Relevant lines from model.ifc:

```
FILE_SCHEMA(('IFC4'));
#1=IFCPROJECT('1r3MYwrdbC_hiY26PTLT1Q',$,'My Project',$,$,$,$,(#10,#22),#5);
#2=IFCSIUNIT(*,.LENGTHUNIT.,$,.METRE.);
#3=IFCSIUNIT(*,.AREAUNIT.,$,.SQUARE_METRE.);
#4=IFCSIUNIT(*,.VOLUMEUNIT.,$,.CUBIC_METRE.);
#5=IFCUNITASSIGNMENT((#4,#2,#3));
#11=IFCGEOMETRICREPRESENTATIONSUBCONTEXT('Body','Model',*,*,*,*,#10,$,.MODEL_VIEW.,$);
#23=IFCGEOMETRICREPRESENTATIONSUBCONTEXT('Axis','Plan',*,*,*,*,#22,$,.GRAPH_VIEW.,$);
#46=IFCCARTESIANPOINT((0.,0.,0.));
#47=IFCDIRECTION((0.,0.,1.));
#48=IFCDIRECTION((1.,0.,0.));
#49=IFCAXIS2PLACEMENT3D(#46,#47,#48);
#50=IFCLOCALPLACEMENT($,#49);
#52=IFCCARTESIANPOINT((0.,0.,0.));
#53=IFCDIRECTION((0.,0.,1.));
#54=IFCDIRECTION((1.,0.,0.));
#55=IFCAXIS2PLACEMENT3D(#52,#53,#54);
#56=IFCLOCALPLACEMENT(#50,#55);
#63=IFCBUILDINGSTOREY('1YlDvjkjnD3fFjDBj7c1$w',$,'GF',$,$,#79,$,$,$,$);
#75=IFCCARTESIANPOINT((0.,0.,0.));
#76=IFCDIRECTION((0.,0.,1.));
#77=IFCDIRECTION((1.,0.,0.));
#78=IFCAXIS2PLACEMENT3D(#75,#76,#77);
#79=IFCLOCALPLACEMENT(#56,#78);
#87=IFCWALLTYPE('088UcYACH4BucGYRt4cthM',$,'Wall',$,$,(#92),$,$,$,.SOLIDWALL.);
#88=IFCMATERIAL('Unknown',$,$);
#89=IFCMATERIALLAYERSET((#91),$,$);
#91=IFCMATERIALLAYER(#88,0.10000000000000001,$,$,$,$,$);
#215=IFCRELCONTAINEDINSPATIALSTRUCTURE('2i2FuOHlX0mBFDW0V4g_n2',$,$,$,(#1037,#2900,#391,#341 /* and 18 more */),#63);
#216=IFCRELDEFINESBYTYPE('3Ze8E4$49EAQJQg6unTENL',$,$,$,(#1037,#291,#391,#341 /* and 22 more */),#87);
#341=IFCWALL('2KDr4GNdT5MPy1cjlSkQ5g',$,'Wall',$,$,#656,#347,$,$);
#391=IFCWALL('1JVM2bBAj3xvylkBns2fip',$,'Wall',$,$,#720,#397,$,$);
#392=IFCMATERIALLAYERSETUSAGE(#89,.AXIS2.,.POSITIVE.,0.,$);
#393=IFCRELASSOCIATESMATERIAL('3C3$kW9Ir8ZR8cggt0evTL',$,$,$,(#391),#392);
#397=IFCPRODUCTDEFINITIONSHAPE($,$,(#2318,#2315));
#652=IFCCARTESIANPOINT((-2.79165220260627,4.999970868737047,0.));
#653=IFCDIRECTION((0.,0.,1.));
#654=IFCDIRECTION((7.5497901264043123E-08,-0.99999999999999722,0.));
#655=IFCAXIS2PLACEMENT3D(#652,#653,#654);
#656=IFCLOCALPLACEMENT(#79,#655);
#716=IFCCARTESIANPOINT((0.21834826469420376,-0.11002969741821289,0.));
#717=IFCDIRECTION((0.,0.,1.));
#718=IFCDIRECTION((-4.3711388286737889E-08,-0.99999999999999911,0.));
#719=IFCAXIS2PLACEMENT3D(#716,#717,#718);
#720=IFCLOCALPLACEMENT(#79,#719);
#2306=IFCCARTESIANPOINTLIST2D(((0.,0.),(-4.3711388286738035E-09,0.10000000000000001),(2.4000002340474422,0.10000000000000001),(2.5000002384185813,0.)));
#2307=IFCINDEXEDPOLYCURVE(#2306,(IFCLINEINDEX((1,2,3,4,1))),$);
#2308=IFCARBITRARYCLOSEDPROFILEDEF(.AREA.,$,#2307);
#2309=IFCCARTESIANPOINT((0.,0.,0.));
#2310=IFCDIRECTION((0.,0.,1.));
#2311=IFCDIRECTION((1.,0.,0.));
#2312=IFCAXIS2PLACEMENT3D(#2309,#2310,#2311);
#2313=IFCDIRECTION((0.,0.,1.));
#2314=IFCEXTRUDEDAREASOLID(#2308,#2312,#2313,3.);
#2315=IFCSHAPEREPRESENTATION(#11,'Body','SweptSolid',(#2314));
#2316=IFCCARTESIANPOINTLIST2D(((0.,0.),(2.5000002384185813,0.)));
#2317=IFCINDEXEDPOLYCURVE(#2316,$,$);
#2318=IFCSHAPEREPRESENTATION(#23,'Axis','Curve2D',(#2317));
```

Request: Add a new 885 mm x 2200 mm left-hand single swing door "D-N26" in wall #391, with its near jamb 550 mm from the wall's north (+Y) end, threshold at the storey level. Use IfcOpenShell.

```python
import numpy as np
import ifcopenshell
import ifcopenshell.api.feature
import ifcopenshell.api.geometry
import ifcopenshell.api.root
import ifcopenshell.api.spatial
import ifcopenshell.geom
import ifcopenshell.util.element
import ifcopenshell.util.placement
import ifcopenshell.util.representation
import ifcopenshell.util.shape
import ifcopenshell.util.unit

model = ifcopenshell.open("model.ifc")
unit_scale = ifcopenshell.util.unit.calculate_unit_scale(model)
settings = ifcopenshell.geom.settings()


def volume(element):
    """Net volume in cubic metres, openings subtracted."""
    shape = ifcopenshell.geom.create_shape(settings, element)
    return ifcopenshell.util.shape.get_volume(shape.geometry)


wall = model.by_guid("1JVM2bBAj3xvylkBns2fip")
storey = ifcopenshell.util.element.get_container(wall, ifc_class="IfcBuildingStorey")
context = ifcopenshell.util.representation.get_context(model, "Model", "Body", "MODEL_VIEW")
before = volume(wall)

width, height, from_end, sill = 0.885, 2.2, 0.55, 0.0  # metres

# The wall runs along its own X axis, and the end named is its -X end.
wall_shape = ifcopenshell.geom.create_shape(settings, wall)
x, y, z = ifcopenshell.util.shape.get_vertices(wall_shape.geometry).T
start = x.min() + from_end
face, thickness = float(y.min()), float(y.max() - y.min())
wall_matrix = ifcopenshell.util.placement.get_local_placement(wall.ObjectPlacement)
level = ifcopenshell.util.placement.get_local_placement(storey.ObjectPlacement)[2, 3]


def in_wall(x, y):
    """Placement at x, y metres in the wall's axes, at sill height."""
    matrix = wall_matrix.copy()
    matrix[:, 3] = wall_matrix @ np.array([x / unit_scale, y / unit_scale, 0.0, 1.0])
    matrix[2, 3] = level + sill / unit_scale
    return matrix


# Opening: a box that overshoots both wall faces by 50 mm.
opening = ifcopenshell.api.root.create_entity(model, ifc_class="IfcOpeningElement", predefined_type="OPENING")
box = ifcopenshell.api.geometry.add_wall_representation(
    model, context=context, length=width, height=height, thickness=thickness + 0.1
)
ifcopenshell.api.geometry.assign_representation(model, product=opening, representation=box)
ifcopenshell.api.geometry.edit_object_placement(model, product=opening, matrix=in_wall(start, face - 0.05), is_si=False)
ifcopenshell.api.feature.add_feature(model, feature=opening, element=wall)

door = ifcopenshell.api.root.create_entity(model, ifc_class="IfcDoor", name="D-N26", predefined_type="DOOR")
door.OverallWidth, door.OverallHeight = width / unit_scale, height / unit_scale
door.OperationType = "SINGLE_SWING_LEFT"
body = ifcopenshell.api.geometry.add_door_representation(
    model,
    context=context,
    overall_width=door.OverallWidth,
    overall_height=door.OverallHeight,
    operation_type="SINGLE_SWING_LEFT",
    lining_properties={"LiningDepth": thickness / unit_scale, "ThresholdDepth": thickness / unit_scale},
)
ifcopenshell.api.geometry.assign_representation(model, product=door, representation=body)
ifcopenshell.api.spatial.assign_container(model, products=[door], relating_structure=storey)
ifcopenshell.api.feature.add_filling(model, opening=opening, element=door)

# The lining spans the wall, so the door starts at the wall face.
ifcopenshell.api.geometry.edit_object_placement(model, product=door, matrix=in_wall(start, face), is_si=False)

after = volume(wall)

print(f"wall volume {before:.3f} -> {after:.3f} m3")

model.write("model_updated.ifc")
```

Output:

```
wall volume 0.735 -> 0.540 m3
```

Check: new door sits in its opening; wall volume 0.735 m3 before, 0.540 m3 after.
